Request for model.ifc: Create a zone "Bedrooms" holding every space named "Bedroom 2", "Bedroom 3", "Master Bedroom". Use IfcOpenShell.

First a look at what the model holds.

```python
import ifcopenshell

model = ifcopenshell.open("model.ifc")
print(model.schema)
seen = {}
for space in model.by_type("IfcSpace"):
    seen[space.LongName] = seen.get(space.LongName, 0) + 1
for name, count in sorted(seen.items(), key=str):
    print(count, "x", name)
print("zones:", [z.Name for z in model.by_type("IfcZone")][:20])
```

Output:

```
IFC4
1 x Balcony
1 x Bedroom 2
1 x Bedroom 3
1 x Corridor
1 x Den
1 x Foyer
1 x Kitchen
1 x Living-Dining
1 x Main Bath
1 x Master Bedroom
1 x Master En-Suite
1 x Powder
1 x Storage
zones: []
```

```python
import ifcopenshell
import ifcopenshell.api.group
import ifcopenshell.api.root

model = ifcopenshell.open("model.ifc")

names = {"Bedroom 2", "Bedroom 3", "Master Bedroom"}
spaces = [s for s in model.by_type("IfcSpace") if s.LongName in names]

zone = ifcopenshell.api.root.create_entity(model, ifc_class="IfcZone", name="Bedrooms")
ifcopenshell.api.group.assign_group(model, products=spaces, group=zone)
print(len(spaces), "spaces in", zone.Name)

model.write("model-out.ifc")
```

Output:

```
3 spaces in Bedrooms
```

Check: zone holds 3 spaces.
